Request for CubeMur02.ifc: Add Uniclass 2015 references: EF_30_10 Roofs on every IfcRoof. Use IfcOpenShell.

First a look at what the model holds.

```python
import ifcopenshell

model = ifcopenshell.open("CubeMur02.ifc")
print(model.schema)
print("classifications:", [c.Name for c in model.by_type("IfcClassification")])
for ifc_class in ("IfcDoor", "IfcRoof", "IfcStair", "IfcWall", "IfcWindow"):
    print(ifc_class, len(model.by_type(ifc_class)))
```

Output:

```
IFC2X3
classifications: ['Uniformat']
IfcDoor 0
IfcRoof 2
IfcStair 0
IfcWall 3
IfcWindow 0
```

```python
import ifcopenshell
import ifcopenshell.api.classification

model = ifcopenshell.open("CubeMur02.ifc")

# IFC2X3 requires Source and Edition and has no link from the project to the system.
system = model.create_entity("IfcClassification", Source="NBS", Edition="2015", Name="Uniclass 2015")

codes = {
    "IfcRoof": ("EF_30_10", "Roofs"),
}
for ifc_class, (code, name) in codes.items():
    products = model.by_type(ifc_class)
    ifcopenshell.api.classification.add_reference(
        model, products=products, classification=system, identification=code, name=name
    )
    print(code, len(products))

model.write("CubeMur02-out.ifc")
```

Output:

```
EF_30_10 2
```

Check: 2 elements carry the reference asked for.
